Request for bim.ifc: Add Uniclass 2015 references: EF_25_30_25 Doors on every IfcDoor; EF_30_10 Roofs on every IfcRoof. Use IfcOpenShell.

First a look at what the model holds.

```python
import ifcopenshell

model = ifcopenshell.open("bim.ifc")
print(model.schema)
print("classifications:", [c.Name for c in model.by_type("IfcClassification")])
for ifc_class in ("IfcDoor", "IfcRoof", "IfcStair", "IfcWall", "IfcWindow"):
    print(ifc_class, len(model.by_type(ifc_class)))
```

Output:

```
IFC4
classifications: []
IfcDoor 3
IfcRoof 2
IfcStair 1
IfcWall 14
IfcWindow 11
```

```python
import ifcopenshell
import ifcopenshell.api.classification

model = ifcopenshell.open("bim.ifc")

system = ifcopenshell.api.classification.add_classification(model, classification="Uniclass 2015")

codes = {
    "IfcDoor": ("EF_25_30_25", "Doors"),
    "IfcRoof": ("EF_30_10", "Roofs"),
}
for ifc_class, (code, name) in codes.items():
    products = model.by_type(ifc_class)
    ifcopenshell.api.classification.add_reference(
        model, products=products, classification=system, identification=code, name=name
    )
    print(code, len(products))

model.write("bim_edited.ifc")
```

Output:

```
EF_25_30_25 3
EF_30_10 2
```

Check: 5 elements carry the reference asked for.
